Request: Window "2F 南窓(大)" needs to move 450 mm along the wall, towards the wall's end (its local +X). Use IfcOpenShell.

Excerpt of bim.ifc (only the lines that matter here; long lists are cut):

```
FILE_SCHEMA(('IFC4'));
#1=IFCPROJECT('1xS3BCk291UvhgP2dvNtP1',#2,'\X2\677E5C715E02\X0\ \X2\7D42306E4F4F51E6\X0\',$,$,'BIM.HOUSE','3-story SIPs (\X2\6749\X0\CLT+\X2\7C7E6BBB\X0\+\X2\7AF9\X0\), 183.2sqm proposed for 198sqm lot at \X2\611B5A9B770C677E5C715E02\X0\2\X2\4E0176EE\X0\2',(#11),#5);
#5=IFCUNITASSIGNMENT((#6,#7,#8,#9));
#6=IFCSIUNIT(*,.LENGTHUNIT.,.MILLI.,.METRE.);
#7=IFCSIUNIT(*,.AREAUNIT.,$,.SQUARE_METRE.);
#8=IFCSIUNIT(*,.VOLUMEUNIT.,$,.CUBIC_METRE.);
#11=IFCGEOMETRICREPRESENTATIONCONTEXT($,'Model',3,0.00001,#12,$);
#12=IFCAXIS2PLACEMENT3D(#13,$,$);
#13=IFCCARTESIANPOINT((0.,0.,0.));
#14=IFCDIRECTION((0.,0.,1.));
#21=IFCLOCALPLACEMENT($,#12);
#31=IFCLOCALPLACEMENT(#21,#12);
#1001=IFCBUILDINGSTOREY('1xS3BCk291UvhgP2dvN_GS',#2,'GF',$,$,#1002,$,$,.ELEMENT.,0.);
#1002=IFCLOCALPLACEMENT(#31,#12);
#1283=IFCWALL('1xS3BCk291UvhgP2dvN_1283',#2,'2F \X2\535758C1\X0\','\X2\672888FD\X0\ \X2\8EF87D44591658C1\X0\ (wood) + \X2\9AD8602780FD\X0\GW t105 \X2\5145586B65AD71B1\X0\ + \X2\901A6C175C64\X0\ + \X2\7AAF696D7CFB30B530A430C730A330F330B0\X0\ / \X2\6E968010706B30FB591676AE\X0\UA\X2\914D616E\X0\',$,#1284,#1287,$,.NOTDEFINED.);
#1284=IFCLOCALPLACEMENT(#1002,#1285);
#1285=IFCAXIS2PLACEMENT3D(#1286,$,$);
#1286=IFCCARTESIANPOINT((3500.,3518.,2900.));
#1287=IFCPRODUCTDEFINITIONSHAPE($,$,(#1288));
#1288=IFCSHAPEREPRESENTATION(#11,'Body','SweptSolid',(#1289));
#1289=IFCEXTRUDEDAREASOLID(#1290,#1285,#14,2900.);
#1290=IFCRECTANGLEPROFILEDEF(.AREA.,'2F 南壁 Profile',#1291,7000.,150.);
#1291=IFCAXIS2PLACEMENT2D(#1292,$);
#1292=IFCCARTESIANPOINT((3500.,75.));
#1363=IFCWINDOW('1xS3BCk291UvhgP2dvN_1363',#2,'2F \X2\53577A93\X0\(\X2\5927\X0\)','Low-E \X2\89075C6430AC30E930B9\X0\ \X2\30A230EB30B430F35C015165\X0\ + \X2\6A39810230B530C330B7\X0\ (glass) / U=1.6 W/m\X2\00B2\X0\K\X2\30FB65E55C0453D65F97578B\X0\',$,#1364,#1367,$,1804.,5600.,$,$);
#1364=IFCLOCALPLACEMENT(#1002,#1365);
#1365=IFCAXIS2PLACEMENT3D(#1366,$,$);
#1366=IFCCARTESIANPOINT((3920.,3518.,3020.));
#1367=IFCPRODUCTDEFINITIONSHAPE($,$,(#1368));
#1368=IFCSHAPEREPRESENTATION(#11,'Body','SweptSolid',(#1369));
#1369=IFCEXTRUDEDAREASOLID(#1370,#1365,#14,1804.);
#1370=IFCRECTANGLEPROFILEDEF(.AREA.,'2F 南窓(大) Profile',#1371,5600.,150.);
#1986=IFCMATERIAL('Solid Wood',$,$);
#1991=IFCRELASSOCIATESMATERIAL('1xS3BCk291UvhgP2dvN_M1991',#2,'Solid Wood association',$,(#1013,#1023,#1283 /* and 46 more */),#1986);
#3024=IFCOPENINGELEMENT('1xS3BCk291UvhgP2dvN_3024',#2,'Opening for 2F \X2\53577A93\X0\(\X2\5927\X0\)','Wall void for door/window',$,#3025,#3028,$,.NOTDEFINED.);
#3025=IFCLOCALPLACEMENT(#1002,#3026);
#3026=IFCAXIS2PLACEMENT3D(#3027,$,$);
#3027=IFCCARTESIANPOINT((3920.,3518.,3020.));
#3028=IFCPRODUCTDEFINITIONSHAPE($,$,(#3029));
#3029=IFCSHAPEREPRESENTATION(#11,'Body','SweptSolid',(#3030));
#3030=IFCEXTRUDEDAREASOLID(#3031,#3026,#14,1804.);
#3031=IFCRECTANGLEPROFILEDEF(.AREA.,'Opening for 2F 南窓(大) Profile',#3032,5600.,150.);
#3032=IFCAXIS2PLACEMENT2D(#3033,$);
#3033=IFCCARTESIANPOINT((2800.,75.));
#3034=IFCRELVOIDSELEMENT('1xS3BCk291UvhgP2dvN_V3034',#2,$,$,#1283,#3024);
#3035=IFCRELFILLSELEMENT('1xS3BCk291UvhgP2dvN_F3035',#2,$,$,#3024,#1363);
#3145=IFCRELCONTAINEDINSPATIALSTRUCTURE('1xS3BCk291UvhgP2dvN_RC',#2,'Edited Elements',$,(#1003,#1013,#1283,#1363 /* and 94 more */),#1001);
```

```python
import ifcopenshell
import ifcopenshell.api.geometry
import ifcopenshell.util.placement
import ifcopenshell.util.unit

model = ifcopenshell.open("bim.ifc")
unit_scale = ifcopenshell.util.unit.calculate_unit_scale(model)

window = model.by_guid("1xS3BCk291UvhgP2dvN_1363")
opening = window.FillsVoids[0].RelatingOpeningElement
wall = opening.VoidsElements[0].RelatingBuildingElement

wall_matrix = ifcopenshell.util.placement.get_local_placement(wall.ObjectPlacement)
shift = wall_matrix[:3, 0] * 0.45 / unit_scale
before = ifcopenshell.util.placement.get_local_placement(window.ObjectPlacement)[:3, 3].copy()

# The window is not placed relative to its opening, so move both.
for product in (opening, window):
    matrix = ifcopenshell.util.placement.get_local_placement(product.ObjectPlacement)
    matrix[:3, 3] += shift
    ifcopenshell.api.geometry.edit_object_placement(model, product=product, matrix=matrix, is_si=False)

after = ifcopenshell.util.placement.get_local_placement(window.ObjectPlacement)[:3, 3]
print("window moved by", (after - before).round(3) + 0.0)

model.write("bim_updated.ifc")
```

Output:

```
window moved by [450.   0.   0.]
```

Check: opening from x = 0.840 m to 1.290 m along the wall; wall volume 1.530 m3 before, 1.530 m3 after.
